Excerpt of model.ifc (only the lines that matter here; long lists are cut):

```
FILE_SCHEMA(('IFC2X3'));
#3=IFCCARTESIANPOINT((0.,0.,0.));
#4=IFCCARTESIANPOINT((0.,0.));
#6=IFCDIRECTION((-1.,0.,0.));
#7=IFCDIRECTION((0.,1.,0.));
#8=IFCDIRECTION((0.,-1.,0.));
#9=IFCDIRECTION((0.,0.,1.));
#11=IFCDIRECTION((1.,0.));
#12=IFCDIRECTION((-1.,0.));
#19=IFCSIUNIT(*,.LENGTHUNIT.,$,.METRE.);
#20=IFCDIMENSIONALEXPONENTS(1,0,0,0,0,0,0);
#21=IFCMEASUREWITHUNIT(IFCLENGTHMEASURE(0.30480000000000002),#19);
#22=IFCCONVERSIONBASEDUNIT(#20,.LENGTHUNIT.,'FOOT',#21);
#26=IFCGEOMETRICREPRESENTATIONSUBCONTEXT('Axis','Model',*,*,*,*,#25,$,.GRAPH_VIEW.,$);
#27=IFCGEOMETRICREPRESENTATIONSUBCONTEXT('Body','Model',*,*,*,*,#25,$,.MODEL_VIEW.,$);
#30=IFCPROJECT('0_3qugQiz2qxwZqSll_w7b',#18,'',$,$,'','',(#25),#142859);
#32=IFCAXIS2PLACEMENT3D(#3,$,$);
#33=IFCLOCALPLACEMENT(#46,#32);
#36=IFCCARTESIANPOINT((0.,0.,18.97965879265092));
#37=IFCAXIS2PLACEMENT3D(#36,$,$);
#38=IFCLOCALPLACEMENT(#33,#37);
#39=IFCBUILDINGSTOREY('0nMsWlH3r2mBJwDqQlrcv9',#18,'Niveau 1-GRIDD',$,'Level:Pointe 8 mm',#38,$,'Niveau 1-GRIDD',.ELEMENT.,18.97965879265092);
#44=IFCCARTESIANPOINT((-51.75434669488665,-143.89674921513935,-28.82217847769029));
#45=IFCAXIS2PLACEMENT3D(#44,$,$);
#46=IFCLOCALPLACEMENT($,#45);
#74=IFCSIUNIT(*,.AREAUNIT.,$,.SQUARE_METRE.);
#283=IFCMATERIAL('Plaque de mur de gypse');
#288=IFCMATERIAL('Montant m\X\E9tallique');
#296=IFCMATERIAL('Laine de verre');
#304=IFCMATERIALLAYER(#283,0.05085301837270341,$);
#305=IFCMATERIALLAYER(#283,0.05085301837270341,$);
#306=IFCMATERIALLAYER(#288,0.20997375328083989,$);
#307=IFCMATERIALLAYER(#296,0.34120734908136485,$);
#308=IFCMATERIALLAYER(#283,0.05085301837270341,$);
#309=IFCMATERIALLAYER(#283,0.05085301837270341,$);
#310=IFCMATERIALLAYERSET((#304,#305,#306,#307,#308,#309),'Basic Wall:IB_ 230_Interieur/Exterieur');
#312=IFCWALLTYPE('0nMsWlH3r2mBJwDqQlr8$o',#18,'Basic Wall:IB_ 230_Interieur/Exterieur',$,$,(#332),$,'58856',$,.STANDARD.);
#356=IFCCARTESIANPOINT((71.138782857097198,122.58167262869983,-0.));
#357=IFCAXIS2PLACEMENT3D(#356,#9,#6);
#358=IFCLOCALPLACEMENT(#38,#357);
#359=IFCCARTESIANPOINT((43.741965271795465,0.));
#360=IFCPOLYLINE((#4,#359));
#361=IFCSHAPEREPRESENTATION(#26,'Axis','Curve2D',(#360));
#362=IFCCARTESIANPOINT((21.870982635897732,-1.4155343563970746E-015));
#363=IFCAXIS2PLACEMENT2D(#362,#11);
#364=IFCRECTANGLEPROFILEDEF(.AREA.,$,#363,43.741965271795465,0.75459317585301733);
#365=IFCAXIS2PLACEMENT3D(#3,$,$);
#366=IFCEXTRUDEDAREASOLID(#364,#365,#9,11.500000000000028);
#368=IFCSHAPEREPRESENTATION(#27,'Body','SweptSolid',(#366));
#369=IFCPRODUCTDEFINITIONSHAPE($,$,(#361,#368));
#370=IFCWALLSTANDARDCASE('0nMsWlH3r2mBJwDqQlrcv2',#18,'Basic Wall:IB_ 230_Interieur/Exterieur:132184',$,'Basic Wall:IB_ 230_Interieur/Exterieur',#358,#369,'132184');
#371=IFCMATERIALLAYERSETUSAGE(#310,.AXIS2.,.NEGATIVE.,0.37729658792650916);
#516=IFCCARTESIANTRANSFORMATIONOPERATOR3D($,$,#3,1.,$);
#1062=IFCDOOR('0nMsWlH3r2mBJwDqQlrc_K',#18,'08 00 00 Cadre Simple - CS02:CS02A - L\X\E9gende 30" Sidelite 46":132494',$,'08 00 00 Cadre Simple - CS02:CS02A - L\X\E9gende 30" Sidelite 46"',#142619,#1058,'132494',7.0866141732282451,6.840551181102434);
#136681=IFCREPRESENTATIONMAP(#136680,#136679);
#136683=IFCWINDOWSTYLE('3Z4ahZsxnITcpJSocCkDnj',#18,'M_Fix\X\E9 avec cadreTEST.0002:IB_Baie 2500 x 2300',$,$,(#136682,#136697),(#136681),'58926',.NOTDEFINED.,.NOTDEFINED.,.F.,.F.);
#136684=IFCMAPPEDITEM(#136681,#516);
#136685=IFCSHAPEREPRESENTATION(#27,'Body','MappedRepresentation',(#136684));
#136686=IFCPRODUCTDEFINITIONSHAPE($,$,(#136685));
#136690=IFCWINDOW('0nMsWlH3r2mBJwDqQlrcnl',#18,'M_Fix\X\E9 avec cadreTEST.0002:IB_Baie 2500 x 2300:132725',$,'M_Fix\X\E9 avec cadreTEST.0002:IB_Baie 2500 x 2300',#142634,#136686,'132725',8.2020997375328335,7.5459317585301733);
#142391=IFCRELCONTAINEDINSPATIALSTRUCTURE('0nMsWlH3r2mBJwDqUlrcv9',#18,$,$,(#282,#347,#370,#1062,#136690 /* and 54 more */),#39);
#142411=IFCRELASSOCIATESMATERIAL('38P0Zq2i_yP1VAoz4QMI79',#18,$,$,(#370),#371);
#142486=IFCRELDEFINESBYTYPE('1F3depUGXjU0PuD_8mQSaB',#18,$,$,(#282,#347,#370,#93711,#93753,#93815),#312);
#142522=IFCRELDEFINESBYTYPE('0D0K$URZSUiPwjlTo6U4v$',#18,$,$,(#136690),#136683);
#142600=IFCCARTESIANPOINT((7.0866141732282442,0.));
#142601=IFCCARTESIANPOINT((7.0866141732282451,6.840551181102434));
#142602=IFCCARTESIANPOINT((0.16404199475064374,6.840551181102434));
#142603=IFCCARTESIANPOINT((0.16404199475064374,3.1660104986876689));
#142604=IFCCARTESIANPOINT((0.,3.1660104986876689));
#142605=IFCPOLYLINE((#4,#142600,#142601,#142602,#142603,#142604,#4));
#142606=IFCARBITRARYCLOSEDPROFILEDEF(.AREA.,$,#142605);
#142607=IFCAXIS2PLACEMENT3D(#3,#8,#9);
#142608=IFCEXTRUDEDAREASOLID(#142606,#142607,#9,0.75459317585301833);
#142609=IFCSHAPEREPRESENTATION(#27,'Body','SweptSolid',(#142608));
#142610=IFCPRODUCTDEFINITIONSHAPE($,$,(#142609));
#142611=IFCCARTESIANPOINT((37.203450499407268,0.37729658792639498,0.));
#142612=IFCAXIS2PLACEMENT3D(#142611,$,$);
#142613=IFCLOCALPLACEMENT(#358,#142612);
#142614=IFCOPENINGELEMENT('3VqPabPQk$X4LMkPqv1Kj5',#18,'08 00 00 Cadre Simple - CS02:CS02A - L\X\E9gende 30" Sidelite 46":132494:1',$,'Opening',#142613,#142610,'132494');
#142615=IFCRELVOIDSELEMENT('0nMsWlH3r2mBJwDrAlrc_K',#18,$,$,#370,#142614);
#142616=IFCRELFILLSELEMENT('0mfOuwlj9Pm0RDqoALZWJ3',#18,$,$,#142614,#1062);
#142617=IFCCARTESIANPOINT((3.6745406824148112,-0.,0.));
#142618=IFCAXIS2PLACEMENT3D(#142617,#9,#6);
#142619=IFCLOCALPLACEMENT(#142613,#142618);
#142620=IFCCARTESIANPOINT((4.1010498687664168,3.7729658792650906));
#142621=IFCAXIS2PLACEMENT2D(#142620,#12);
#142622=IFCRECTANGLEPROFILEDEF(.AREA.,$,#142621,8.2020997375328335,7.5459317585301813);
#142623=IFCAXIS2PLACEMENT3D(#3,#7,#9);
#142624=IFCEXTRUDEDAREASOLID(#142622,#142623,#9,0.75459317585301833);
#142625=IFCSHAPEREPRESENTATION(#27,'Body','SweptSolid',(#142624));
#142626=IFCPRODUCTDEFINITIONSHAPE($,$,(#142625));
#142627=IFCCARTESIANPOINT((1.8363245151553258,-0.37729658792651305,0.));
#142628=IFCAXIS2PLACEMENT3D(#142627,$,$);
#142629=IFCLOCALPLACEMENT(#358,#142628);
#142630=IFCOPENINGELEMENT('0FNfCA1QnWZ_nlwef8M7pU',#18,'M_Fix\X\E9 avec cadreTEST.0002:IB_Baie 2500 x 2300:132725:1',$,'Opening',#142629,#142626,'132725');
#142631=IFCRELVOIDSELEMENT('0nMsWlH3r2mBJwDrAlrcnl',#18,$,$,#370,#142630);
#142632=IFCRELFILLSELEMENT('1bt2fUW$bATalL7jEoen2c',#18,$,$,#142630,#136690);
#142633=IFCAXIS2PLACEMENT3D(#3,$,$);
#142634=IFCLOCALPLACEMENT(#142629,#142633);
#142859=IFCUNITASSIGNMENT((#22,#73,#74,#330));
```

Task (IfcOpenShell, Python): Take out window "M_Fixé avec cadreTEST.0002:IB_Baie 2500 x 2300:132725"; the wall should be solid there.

```python
import ifcopenshell
import ifcopenshell.api.feature
import ifcopenshell.api.root
import ifcopenshell.geom
import ifcopenshell.util.shape

model = ifcopenshell.open("model.ifc")
settings = ifcopenshell.geom.settings()


def volume(element):
    """Net volume in cubic metres, openings subtracted."""
    shape = ifcopenshell.geom.create_shape(settings, element)
    return ifcopenshell.util.shape.get_volume(shape.geometry)


window = model.by_guid("0nMsWlH3r2mBJwDqQlrcnl")
opening = window.FillsVoids[0].RelatingOpeningElement
wall = opening.VoidsElements[0].RelatingBuildingElement
before = volume(wall)

ifcopenshell.api.root.remove_product(model, product=window)
ifcopenshell.api.feature.remove_feature(model, feature=opening)

after = volume(wall)

print(f"wall volume {before:.3f} -> {after:.3f} m3")

model.write("model_rev.ifc")
```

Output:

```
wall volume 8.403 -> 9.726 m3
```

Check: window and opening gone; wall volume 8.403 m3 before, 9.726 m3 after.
